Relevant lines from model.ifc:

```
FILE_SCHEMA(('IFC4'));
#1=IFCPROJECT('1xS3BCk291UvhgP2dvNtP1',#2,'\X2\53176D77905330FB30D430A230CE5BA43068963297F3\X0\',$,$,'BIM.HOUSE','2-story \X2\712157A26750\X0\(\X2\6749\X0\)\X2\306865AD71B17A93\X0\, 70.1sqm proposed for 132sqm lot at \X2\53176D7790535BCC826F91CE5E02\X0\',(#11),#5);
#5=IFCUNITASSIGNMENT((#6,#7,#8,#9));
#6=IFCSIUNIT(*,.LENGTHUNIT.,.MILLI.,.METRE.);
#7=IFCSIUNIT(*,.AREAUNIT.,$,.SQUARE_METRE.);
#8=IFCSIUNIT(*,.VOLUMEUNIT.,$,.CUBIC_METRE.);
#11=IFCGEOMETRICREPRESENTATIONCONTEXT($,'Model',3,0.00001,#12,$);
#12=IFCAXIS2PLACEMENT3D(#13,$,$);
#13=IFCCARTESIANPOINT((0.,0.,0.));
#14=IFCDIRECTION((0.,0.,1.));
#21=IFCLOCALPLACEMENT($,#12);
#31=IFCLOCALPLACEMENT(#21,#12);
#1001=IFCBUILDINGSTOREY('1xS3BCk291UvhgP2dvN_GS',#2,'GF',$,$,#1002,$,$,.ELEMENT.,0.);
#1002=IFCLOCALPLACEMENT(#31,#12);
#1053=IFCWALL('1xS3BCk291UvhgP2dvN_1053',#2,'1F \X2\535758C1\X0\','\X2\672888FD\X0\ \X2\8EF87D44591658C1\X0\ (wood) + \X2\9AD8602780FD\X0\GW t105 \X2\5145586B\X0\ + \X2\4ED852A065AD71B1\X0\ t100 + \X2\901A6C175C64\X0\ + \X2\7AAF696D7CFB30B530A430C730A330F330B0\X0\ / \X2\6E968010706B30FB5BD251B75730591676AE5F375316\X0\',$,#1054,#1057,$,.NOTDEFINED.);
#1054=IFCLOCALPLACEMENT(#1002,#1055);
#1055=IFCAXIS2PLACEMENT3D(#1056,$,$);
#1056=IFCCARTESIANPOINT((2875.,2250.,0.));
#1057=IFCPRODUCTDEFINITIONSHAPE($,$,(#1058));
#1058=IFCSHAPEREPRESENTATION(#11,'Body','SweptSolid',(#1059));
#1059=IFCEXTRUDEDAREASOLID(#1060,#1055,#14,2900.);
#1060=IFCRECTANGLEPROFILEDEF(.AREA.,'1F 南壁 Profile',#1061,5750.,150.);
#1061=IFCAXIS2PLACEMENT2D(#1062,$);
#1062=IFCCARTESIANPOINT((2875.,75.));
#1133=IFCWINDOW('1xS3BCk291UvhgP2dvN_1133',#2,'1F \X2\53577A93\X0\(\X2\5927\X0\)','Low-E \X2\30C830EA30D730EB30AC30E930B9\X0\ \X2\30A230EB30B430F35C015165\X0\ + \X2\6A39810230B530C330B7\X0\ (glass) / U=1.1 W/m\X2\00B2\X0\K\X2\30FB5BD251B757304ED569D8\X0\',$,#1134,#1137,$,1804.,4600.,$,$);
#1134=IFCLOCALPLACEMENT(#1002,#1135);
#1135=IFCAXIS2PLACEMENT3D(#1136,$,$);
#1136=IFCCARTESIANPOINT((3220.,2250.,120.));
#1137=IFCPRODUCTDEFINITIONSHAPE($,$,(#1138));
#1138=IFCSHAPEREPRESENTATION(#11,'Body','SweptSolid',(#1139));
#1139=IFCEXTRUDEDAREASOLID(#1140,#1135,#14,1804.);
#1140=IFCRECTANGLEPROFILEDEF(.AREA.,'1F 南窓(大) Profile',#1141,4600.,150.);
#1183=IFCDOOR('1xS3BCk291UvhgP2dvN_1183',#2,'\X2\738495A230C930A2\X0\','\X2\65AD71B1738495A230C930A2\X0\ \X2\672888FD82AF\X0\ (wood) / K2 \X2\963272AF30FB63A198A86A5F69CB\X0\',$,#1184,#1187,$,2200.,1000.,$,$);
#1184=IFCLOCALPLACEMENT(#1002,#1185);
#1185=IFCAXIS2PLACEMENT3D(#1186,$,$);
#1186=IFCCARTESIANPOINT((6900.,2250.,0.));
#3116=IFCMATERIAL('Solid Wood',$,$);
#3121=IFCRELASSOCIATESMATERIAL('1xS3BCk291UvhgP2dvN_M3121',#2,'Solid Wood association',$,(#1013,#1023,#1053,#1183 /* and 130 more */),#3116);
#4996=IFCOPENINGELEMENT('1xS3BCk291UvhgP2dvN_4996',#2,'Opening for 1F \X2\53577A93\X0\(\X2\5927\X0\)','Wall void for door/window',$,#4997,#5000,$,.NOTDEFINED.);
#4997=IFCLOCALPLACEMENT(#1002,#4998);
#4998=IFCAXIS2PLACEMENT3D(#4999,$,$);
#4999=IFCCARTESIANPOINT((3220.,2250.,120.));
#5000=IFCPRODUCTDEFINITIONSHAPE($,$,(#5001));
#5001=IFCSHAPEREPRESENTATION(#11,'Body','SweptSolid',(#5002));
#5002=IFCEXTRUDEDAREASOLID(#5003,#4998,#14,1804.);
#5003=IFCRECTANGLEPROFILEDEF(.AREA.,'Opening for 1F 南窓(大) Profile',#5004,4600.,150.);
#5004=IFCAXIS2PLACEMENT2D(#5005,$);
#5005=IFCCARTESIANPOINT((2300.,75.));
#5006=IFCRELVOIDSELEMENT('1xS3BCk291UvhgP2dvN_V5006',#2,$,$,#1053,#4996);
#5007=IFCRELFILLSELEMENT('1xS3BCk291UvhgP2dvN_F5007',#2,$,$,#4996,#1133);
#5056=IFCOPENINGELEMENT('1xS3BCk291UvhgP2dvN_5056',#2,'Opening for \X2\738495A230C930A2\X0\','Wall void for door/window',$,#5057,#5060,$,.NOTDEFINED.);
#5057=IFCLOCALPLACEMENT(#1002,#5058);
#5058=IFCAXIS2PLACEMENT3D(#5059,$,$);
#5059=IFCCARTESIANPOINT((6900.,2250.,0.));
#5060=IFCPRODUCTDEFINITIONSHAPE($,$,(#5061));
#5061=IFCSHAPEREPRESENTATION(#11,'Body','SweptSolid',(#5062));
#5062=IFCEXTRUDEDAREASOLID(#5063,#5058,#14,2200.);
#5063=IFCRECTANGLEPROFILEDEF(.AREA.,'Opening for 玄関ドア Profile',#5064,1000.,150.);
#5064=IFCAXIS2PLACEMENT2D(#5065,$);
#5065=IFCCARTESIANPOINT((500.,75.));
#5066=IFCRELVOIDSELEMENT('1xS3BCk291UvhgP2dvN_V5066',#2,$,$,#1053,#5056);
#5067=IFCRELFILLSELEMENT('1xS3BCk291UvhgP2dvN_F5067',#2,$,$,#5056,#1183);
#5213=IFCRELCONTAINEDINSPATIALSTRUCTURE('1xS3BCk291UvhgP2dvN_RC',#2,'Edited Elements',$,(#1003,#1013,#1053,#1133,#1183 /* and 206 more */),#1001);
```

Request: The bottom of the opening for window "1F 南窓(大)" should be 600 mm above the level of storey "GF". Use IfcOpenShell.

```python
import numpy as np
import ifcopenshell
import ifcopenshell.api.geometry
import ifcopenshell.geom
import ifcopenshell.util.element
import ifcopenshell.util.placement
import ifcopenshell.util.shape
import ifcopenshell.util.unit

model = ifcopenshell.open("model.ifc")
unit_scale = ifcopenshell.util.unit.calculate_unit_scale(model)

window = model.by_guid("1xS3BCk291UvhgP2dvN_1133")
opening = window.FillsVoids[0].RelatingOpeningElement
storey = ifcopenshell.util.element.get_container(window, ifc_class="IfcBuildingStorey")
level = ifcopenshell.util.placement.get_local_placement(storey.ObjectPlacement)[2, 3]

# The opening's origin need not be at the sill, so measure its lowest point.
shape = ifcopenshell.geom.create_shape(ifcopenshell.geom.settings(), opening)
bottom = ifcopenshell.util.shape.get_shape_bottom_elevation(shape, shape.geometry) / unit_scale
dz = level + 0.6 / unit_scale - bottom

shift = np.array([0.0, 0.0, dz])
# The window is not placed relative to its opening, so move both.
for product in (opening, window):
    matrix = ifcopenshell.util.placement.get_local_placement(product.ObjectPlacement)
    matrix[:3, 3] += shift
    ifcopenshell.api.geometry.edit_object_placement(model, product=product, matrix=matrix, is_si=False)

print(f"moved by {dz * unit_scale:+.3f} m")

model.write("model_rev.ifc")
```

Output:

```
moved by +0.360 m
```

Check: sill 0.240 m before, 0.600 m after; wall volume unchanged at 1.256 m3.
